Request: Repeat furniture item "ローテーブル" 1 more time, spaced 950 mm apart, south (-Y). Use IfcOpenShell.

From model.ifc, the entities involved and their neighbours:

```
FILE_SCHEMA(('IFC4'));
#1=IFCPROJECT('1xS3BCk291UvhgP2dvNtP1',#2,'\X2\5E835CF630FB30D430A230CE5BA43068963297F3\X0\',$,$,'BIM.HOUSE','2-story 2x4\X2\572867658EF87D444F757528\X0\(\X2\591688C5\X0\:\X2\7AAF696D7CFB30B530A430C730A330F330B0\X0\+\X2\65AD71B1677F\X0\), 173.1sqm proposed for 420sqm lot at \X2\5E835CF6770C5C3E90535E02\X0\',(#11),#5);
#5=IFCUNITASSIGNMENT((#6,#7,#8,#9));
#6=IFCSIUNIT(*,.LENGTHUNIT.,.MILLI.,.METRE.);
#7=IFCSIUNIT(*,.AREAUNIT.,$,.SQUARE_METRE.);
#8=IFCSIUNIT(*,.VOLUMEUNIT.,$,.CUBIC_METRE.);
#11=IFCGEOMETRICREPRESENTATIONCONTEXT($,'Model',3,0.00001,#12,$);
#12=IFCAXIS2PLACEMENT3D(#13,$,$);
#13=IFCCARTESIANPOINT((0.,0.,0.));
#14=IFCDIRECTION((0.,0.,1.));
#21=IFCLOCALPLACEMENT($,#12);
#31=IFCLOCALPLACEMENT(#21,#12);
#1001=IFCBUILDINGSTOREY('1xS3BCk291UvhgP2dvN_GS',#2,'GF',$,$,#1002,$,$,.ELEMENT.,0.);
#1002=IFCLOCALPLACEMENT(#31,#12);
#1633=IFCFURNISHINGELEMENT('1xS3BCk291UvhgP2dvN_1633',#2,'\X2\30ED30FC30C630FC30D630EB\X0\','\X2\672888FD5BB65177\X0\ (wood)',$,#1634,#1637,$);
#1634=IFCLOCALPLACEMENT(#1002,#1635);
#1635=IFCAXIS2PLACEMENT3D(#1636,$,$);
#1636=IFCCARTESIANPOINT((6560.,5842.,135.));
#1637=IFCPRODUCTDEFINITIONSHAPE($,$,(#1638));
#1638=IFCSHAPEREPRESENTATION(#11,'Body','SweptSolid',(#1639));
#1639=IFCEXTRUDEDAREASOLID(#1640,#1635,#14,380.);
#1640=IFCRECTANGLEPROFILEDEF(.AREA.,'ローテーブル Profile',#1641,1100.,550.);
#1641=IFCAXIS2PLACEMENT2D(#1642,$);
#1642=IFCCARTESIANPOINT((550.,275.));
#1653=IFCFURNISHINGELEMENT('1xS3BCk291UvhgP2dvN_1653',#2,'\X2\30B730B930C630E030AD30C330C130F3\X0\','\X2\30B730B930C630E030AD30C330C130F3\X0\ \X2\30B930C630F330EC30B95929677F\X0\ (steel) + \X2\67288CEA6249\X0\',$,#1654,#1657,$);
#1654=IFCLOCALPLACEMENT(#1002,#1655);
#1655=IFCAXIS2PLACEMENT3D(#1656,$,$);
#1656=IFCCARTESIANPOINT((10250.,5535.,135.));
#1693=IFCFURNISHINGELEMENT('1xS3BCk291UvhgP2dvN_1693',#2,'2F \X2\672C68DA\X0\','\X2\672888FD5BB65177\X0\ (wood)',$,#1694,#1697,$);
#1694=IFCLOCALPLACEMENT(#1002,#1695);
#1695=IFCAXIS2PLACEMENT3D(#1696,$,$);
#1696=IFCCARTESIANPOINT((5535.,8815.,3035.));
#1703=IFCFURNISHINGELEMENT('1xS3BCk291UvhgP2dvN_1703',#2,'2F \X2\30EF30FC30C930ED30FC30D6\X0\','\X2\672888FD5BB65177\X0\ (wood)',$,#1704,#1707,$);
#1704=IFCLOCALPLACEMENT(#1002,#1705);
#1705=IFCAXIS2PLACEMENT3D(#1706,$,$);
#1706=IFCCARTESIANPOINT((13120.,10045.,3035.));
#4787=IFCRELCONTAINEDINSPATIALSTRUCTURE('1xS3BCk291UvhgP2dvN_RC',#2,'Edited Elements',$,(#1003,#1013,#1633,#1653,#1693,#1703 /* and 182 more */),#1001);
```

```python
import numpy as np
import ifcopenshell
import ifcopenshell.api.geometry
import ifcopenshell.api.root
import ifcopenshell.util.element
import ifcopenshell.util.placement

model = ifcopenshell.open("model.ifc")


def reuse_history(source, copy):
    """copy_class also copies each property set's owner history, people and application; keep the originals."""
    for rel in copy.IsDefinedBy:
        if rel.is_a("IfcRelDefinesByProperties") and (history := rel.RelatingPropertyDefinition.OwnerHistory):
            rel.RelatingPropertyDefinition.OwnerHistory = source.OwnerHistory
            ifcopenshell.util.element.remove_deep2(model, history)


source = model.by_guid("1xS3BCk291UvhgP2dvN_1633")
base = ifcopenshell.util.placement.get_local_placement(source.ObjectPlacement)
step = np.array([0.0, -1.0, 0.0]) * 950.0

for i in range(1, 2):
    copy = ifcopenshell.api.root.copy_class(model, product=source)
    copy.Representation = ifcopenshell.util.element.copy_deep(
        model, source.Representation, exclude=["IfcGeometricRepresentationContext", "IfcRepresentationMap"]
    )
    reuse_history(source, copy)
    matrix = base.copy()
    matrix[:3, 3] += i * step
    print("added at", matrix[:3, 3].round(3) + 0.0)
    ifcopenshell.api.geometry.edit_object_placement(model, product=copy, matrix=matrix, is_si=False)

model.write("model_edited.ifc")
```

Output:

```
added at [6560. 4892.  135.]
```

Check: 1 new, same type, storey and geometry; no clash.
